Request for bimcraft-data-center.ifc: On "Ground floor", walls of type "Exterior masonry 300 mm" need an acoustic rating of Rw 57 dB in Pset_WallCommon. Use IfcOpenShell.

First a look at what the model holds.

```python
import ifcopenshell
import ifcopenshell.util.element

model = ifcopenshell.open("bimcraft-data-center.ifc")
print(model.schema)
storey = next(s for s in model.by_type("IfcBuildingStorey") if s.Name == "Ground floor")
walls = [e for e in ifcopenshell.util.element.get_decomposition(storey) if e.is_a("IfcWall")]
seen = {}
for e in walls:
    element_type = ifcopenshell.util.element.get_type(e)
    key = (element_type.Name if element_type != e and element_type else None, ifcopenshell.util.element.get_pset(e, "Pset_WallCommon", "AcousticRating"))
    seen[key] = seen.get(key, 0) + 1
for (name, value), count in sorted(seen.items(), key=str):
    print(count, "x", name, "|", value)
```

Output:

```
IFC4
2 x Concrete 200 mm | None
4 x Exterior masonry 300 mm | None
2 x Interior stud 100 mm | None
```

```python
import ifcopenshell
import ifcopenshell.api.pset
import ifcopenshell.util.element

model = ifcopenshell.open("bimcraft-data-center.ifc")

storey = next(s for s in model.by_type("IfcBuildingStorey") if s.Name == "Ground floor")
walls = [e for e in ifcopenshell.util.element.get_decomposition(storey) if e.is_a("IfcWall")]

count = 0
for e in walls:
    element_type = ifcopenshell.util.element.get_type(e)
    if element_type in (None, e) or element_type.Name != "Exterior masonry 300 mm":
        continue
    # add_pset returns the element's existing set when there is one.
    pset = ifcopenshell.api.pset.add_pset(model, product=e, name="Pset_WallCommon")
    ifcopenshell.api.pset.edit_pset(model, pset=pset, properties={"AcousticRating": "Rw 57 dB"})
    count += 1

print(count, "walls updated")

model.write("bimcraft-data-center_edited.ifc")
```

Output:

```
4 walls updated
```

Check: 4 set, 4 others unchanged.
